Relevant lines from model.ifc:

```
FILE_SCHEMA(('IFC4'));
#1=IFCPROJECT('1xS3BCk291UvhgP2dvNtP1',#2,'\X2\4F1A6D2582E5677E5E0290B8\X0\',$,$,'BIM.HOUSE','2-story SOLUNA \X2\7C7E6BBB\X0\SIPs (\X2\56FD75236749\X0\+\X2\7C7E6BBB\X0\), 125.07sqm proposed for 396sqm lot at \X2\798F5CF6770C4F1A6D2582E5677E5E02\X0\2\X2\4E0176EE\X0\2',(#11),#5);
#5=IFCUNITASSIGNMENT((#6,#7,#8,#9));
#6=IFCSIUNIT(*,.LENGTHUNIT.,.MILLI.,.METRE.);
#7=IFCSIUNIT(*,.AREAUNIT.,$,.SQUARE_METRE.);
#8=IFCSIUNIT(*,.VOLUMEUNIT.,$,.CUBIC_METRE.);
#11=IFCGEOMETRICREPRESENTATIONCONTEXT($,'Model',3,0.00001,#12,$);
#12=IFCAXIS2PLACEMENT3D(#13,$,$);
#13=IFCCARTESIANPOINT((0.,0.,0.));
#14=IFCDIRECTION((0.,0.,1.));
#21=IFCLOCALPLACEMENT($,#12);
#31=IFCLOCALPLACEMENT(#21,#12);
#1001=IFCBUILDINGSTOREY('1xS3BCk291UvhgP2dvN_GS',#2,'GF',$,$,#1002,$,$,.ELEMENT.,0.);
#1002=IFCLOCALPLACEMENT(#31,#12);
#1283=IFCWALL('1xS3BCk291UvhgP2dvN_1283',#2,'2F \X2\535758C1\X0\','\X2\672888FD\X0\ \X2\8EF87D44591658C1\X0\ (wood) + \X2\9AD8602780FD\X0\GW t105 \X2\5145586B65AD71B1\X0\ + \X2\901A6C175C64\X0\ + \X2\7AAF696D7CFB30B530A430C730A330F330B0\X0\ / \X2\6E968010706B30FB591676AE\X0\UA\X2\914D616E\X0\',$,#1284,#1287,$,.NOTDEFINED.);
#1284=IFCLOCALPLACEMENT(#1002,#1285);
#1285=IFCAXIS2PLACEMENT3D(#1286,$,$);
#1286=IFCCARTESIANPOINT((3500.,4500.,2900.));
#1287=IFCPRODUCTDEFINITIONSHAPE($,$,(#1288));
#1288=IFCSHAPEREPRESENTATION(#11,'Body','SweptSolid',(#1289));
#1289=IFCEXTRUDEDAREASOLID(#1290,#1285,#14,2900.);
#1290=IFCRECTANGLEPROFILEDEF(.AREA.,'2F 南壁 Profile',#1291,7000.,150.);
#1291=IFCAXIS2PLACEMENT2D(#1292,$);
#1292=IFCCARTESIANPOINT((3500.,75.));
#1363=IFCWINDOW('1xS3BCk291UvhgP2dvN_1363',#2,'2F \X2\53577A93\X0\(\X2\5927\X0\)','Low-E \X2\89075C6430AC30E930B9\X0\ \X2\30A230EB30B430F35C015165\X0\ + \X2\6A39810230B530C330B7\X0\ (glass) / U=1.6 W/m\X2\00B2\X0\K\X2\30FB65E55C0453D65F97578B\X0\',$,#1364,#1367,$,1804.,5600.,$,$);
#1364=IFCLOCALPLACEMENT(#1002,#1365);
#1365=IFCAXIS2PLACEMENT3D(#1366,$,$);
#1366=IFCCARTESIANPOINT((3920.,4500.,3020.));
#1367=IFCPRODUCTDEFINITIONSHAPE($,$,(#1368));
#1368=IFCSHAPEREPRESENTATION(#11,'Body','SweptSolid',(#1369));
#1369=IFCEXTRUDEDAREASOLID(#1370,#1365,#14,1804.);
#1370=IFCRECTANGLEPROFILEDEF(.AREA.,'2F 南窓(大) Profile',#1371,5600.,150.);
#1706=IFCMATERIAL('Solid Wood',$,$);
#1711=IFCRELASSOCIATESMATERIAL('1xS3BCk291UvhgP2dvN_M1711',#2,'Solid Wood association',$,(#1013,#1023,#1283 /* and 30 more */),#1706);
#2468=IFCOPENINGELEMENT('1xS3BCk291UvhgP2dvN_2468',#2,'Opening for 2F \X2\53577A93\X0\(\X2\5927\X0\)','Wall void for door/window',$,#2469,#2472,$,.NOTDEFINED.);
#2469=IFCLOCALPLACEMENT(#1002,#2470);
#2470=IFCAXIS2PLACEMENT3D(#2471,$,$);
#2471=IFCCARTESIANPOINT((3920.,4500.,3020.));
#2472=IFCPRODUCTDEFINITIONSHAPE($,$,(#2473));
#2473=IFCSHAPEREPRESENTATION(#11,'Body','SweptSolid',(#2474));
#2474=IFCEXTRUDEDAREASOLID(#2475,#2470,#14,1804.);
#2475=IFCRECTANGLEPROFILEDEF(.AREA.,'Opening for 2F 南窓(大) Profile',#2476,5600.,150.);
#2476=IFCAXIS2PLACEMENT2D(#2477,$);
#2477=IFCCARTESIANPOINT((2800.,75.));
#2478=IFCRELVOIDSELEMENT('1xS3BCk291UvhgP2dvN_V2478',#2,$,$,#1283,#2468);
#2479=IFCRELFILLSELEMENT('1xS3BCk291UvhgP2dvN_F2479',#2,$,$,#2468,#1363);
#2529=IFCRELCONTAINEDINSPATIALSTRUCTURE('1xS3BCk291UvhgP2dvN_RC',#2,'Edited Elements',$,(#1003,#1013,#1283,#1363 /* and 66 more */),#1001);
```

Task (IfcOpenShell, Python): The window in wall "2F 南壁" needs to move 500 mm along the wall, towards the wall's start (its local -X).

```python
import ifcopenshell
import ifcopenshell.api.geometry
import ifcopenshell.util.placement
import ifcopenshell.util.unit

model = ifcopenshell.open("model.ifc")
unit_scale = ifcopenshell.util.unit.calculate_unit_scale(model)

window = model.by_guid("1xS3BCk291UvhgP2dvN_1363")
opening = window.FillsVoids[0].RelatingOpeningElement
wall = opening.VoidsElements[0].RelatingBuildingElement

wall_matrix = ifcopenshell.util.placement.get_local_placement(wall.ObjectPlacement)
shift = wall_matrix[:3, 0] * -0.5 / unit_scale
before = ifcopenshell.util.placement.get_local_placement(window.ObjectPlacement)[:3, 3].copy()

# The window is not placed relative to its opening, so move both.
for product in (opening, window):
    matrix = ifcopenshell.util.placement.get_local_placement(product.ObjectPlacement)
    matrix[:3, 3] += shift
    ifcopenshell.api.geometry.edit_object_placement(model, product=product, matrix=matrix, is_si=False)

after = ifcopenshell.util.placement.get_local_placement(window.ObjectPlacement)[:3, 3]
print("window moved by", (after - before).round(3) + 0.0)

model.write("model_updated.ifc")
```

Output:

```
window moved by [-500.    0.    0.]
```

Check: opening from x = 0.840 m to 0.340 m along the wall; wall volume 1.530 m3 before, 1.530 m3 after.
